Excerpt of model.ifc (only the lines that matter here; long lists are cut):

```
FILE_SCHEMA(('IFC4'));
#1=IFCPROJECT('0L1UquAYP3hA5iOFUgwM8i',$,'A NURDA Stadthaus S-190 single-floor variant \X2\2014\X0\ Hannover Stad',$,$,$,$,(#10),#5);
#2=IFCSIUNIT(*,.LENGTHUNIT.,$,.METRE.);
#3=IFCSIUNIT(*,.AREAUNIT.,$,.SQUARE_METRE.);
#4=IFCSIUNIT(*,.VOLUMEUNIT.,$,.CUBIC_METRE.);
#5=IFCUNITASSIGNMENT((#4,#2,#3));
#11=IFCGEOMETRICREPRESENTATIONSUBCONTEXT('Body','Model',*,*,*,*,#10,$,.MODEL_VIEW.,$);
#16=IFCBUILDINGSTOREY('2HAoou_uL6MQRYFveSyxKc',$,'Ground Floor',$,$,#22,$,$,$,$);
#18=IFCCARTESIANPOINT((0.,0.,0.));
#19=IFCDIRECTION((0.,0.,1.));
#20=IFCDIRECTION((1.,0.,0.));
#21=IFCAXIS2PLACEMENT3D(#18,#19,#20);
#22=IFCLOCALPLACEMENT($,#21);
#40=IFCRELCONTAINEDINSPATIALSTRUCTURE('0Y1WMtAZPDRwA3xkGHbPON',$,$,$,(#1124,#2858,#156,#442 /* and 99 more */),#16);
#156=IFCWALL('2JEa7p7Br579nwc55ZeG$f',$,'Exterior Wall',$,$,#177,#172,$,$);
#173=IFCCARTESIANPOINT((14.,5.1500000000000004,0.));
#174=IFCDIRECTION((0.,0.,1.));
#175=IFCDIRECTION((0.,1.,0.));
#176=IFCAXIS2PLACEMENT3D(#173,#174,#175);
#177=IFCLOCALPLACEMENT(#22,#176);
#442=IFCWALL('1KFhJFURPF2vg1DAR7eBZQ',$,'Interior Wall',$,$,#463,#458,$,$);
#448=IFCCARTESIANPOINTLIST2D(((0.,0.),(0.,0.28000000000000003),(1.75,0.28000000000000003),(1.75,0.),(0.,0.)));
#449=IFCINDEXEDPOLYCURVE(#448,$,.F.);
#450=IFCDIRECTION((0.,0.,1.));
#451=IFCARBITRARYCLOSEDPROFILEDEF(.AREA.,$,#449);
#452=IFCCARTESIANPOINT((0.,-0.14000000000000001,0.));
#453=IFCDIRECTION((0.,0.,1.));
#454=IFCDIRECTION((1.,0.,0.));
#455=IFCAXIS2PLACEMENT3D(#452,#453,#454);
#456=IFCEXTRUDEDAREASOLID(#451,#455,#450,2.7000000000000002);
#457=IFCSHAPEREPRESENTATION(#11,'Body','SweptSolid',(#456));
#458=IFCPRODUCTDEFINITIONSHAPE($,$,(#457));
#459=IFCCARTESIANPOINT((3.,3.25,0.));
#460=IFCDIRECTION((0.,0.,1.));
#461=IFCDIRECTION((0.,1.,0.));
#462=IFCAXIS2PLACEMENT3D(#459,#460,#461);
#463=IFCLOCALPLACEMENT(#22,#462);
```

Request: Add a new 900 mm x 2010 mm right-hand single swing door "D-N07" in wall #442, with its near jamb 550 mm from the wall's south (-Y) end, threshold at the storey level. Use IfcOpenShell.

```python
import numpy as np
import ifcopenshell
import ifcopenshell.api.feature
import ifcopenshell.api.geometry
import ifcopenshell.api.root
import ifcopenshell.api.spatial
import ifcopenshell.geom
import ifcopenshell.util.element
import ifcopenshell.util.placement
import ifcopenshell.util.representation
import ifcopenshell.util.shape
import ifcopenshell.util.unit

model = ifcopenshell.open("model.ifc")
unit_scale = ifcopenshell.util.unit.calculate_unit_scale(model)
settings = ifcopenshell.geom.settings()


def volume(element):
    """Net volume in cubic metres, openings subtracted."""
    shape = ifcopenshell.geom.create_shape(settings, element)
    return ifcopenshell.util.shape.get_volume(shape.geometry)


wall = model.by_guid("1KFhJFURPF2vg1DAR7eBZQ")
storey = ifcopenshell.util.element.get_container(wall, ifc_class="IfcBuildingStorey")
context = ifcopenshell.util.representation.get_context(model, "Model", "Body", "MODEL_VIEW")
before = volume(wall)

width, height, from_end, sill = 0.9, 2.01, 0.55, 0.0  # metres

# The wall runs along its own X axis, and the end named is its -X end.
wall_shape = ifcopenshell.geom.create_shape(settings, wall)
x, y, z = ifcopenshell.util.shape.get_vertices(wall_shape.geometry).T
start = x.min() + from_end
face, thickness = float(y.min()), float(y.max() - y.min())
wall_matrix = ifcopenshell.util.placement.get_local_placement(wall.ObjectPlacement)
level = ifcopenshell.util.placement.get_local_placement(storey.ObjectPlacement)[2, 3]


def in_wall(x, y):
    """Placement at x, y metres in the wall's axes, at sill height."""
    matrix = wall_matrix.copy()
    matrix[:, 3] = wall_matrix @ np.array([x / unit_scale, y / unit_scale, 0.0, 1.0])
    matrix[2, 3] = level + sill / unit_scale
    return matrix


# Opening: a box that overshoots both wall faces by 50 mm.
opening = ifcopenshell.api.root.create_entity(model, ifc_class="IfcOpeningElement", predefined_type="OPENING")
box = ifcopenshell.api.geometry.add_wall_representation(
    model, context=context, length=width, height=height, thickness=thickness + 0.1
)
ifcopenshell.api.geometry.assign_representation(model, product=opening, representation=box)
ifcopenshell.api.geometry.edit_object_placement(model, product=opening, matrix=in_wall(start, face - 0.05), is_si=False)
ifcopenshell.api.feature.add_feature(model, feature=opening, element=wall)

door = ifcopenshell.api.root.create_entity(model, ifc_class="IfcDoor", name="D-N07", predefined_type="DOOR")
door.OverallWidth, door.OverallHeight = width / unit_scale, height / unit_scale
door.OperationType = "SINGLE_SWING_RIGHT"
body = ifcopenshell.api.geometry.add_door_representation(
    model,
    context=context,
    overall_width=door.OverallWidth,
    overall_height=door.OverallHeight,
    operation_type="SINGLE_SWING_RIGHT",
    lining_properties={"LiningDepth": thickness / unit_scale, "ThresholdDepth": thickness / unit_scale},
)
ifcopenshell.api.geometry.assign_representation(model, product=door, representation=body)
ifcopenshell.api.spatial.assign_container(model, products=[door], relating_structure=storey)
ifcopenshell.api.feature.add_filling(model, opening=opening, element=door)

# The lining spans the wall, so the door starts at the wall face.
ifcopenshell.api.geometry.edit_object_placement(model, product=door, matrix=in_wall(start, face), is_si=False)

after = volume(wall)

print(f"wall volume {before:.3f} -> {after:.3f} m3")

model.write("model_updated.ifc")
```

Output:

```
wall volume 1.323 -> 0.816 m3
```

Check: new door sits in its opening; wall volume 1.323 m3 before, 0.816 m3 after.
